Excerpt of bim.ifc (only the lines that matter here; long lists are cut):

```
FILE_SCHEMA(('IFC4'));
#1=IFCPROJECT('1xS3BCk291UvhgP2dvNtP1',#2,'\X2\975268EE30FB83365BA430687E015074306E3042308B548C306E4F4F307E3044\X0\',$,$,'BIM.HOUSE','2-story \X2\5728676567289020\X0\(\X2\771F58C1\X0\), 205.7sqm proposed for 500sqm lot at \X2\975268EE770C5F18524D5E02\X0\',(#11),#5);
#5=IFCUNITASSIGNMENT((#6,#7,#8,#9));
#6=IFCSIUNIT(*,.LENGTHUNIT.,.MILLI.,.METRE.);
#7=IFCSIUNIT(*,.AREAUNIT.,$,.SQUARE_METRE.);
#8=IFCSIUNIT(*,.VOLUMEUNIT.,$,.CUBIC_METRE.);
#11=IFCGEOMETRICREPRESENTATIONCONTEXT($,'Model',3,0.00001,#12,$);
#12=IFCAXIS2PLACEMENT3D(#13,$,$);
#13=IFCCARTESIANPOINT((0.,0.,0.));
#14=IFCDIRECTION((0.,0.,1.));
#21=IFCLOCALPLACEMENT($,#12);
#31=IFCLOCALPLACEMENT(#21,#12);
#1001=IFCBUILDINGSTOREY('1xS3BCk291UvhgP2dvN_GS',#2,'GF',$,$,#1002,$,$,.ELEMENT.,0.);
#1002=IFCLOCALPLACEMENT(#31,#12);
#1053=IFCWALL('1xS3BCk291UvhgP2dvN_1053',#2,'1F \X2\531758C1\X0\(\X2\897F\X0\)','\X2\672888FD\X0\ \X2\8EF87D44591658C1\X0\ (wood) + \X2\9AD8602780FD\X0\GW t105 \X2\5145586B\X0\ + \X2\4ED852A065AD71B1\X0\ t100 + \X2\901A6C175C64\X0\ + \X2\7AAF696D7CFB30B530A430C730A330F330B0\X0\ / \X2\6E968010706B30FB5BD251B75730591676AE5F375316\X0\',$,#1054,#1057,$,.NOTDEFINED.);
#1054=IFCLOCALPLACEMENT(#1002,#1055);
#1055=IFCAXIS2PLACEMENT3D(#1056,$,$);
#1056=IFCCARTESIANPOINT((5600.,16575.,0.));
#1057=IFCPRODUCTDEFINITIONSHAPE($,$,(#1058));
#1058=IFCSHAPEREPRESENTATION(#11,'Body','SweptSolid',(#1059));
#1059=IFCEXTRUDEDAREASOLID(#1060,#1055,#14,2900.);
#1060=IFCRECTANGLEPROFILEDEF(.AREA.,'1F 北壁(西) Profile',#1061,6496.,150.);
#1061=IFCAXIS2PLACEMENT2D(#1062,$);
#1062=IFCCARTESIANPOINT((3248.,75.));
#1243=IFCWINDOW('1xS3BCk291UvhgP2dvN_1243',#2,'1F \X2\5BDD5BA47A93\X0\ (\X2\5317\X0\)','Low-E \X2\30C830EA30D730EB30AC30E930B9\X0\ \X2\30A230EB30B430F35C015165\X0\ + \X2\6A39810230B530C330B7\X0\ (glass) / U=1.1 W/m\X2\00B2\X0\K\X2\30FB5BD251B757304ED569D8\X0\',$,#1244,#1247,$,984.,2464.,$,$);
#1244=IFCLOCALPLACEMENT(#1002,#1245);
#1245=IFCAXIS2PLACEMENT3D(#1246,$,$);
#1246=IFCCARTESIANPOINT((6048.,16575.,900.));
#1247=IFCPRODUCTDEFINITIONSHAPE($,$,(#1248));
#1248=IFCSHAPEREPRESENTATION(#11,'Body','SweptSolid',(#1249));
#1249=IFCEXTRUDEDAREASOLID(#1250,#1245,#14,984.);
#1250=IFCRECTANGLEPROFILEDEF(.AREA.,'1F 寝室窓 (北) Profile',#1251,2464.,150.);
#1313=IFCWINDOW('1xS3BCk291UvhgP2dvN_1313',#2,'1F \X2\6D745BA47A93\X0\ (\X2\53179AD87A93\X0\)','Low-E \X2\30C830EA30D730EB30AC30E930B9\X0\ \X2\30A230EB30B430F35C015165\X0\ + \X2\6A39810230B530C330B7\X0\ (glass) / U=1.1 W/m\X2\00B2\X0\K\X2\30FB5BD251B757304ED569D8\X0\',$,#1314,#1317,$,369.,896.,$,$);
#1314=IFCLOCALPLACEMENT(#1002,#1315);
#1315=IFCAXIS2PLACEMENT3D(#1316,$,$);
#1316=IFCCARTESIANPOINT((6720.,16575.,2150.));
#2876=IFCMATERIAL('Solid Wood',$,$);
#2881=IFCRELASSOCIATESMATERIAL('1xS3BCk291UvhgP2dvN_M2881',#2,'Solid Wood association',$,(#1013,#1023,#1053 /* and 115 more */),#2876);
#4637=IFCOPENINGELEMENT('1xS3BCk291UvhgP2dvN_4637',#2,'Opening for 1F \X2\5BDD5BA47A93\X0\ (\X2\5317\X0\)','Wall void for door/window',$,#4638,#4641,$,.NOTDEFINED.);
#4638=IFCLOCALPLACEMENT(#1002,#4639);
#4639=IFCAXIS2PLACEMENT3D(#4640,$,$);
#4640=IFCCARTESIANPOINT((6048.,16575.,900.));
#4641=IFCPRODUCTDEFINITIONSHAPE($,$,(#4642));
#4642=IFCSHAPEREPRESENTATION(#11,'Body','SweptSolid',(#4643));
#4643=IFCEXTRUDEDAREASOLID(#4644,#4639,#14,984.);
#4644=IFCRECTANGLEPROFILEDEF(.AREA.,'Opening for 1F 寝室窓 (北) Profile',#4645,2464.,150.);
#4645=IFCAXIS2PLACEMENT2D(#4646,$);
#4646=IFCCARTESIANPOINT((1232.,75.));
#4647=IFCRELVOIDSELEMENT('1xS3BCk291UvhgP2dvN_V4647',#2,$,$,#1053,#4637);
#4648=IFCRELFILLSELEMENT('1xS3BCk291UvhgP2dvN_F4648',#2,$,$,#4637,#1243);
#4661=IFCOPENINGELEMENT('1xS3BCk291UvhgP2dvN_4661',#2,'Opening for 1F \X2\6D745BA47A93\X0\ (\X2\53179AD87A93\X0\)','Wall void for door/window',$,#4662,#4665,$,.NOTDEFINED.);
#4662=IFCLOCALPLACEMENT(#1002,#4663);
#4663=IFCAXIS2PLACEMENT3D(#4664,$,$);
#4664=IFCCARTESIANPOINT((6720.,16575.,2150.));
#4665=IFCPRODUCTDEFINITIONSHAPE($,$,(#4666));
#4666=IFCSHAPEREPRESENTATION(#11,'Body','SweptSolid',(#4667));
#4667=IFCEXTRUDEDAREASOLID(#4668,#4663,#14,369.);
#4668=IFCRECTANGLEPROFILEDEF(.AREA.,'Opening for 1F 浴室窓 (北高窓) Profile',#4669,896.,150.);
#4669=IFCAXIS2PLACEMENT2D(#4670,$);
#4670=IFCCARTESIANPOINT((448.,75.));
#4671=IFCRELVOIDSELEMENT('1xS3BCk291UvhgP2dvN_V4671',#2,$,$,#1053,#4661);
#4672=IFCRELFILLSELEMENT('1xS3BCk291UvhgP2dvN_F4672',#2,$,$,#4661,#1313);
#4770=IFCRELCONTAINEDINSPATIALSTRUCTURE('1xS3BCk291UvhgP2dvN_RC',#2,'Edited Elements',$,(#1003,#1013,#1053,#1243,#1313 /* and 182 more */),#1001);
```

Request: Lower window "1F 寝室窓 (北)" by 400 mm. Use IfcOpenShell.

```python
import numpy as np
import ifcopenshell
import ifcopenshell.api.geometry
import ifcopenshell.util.placement
import ifcopenshell.util.unit

model = ifcopenshell.open("bim.ifc")
unit_scale = ifcopenshell.util.unit.calculate_unit_scale(model)

window = model.by_guid("1xS3BCk291UvhgP2dvN_1243")
opening = window.FillsVoids[0].RelatingOpeningElement
dz = -0.4 / unit_scale

shift = np.array([0.0, 0.0, dz])
# The window is not placed relative to its opening, so move both.
for product in (opening, window):
    matrix = ifcopenshell.util.placement.get_local_placement(product.ObjectPlacement)
    matrix[:3, 3] += shift
    ifcopenshell.api.geometry.edit_object_placement(model, product=product, matrix=matrix, is_si=False)

print(f"moved by {dz * unit_scale:+.3f} m")

model.write("bim_rev.ifc")
```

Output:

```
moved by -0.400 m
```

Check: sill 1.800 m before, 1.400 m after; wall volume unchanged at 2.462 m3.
